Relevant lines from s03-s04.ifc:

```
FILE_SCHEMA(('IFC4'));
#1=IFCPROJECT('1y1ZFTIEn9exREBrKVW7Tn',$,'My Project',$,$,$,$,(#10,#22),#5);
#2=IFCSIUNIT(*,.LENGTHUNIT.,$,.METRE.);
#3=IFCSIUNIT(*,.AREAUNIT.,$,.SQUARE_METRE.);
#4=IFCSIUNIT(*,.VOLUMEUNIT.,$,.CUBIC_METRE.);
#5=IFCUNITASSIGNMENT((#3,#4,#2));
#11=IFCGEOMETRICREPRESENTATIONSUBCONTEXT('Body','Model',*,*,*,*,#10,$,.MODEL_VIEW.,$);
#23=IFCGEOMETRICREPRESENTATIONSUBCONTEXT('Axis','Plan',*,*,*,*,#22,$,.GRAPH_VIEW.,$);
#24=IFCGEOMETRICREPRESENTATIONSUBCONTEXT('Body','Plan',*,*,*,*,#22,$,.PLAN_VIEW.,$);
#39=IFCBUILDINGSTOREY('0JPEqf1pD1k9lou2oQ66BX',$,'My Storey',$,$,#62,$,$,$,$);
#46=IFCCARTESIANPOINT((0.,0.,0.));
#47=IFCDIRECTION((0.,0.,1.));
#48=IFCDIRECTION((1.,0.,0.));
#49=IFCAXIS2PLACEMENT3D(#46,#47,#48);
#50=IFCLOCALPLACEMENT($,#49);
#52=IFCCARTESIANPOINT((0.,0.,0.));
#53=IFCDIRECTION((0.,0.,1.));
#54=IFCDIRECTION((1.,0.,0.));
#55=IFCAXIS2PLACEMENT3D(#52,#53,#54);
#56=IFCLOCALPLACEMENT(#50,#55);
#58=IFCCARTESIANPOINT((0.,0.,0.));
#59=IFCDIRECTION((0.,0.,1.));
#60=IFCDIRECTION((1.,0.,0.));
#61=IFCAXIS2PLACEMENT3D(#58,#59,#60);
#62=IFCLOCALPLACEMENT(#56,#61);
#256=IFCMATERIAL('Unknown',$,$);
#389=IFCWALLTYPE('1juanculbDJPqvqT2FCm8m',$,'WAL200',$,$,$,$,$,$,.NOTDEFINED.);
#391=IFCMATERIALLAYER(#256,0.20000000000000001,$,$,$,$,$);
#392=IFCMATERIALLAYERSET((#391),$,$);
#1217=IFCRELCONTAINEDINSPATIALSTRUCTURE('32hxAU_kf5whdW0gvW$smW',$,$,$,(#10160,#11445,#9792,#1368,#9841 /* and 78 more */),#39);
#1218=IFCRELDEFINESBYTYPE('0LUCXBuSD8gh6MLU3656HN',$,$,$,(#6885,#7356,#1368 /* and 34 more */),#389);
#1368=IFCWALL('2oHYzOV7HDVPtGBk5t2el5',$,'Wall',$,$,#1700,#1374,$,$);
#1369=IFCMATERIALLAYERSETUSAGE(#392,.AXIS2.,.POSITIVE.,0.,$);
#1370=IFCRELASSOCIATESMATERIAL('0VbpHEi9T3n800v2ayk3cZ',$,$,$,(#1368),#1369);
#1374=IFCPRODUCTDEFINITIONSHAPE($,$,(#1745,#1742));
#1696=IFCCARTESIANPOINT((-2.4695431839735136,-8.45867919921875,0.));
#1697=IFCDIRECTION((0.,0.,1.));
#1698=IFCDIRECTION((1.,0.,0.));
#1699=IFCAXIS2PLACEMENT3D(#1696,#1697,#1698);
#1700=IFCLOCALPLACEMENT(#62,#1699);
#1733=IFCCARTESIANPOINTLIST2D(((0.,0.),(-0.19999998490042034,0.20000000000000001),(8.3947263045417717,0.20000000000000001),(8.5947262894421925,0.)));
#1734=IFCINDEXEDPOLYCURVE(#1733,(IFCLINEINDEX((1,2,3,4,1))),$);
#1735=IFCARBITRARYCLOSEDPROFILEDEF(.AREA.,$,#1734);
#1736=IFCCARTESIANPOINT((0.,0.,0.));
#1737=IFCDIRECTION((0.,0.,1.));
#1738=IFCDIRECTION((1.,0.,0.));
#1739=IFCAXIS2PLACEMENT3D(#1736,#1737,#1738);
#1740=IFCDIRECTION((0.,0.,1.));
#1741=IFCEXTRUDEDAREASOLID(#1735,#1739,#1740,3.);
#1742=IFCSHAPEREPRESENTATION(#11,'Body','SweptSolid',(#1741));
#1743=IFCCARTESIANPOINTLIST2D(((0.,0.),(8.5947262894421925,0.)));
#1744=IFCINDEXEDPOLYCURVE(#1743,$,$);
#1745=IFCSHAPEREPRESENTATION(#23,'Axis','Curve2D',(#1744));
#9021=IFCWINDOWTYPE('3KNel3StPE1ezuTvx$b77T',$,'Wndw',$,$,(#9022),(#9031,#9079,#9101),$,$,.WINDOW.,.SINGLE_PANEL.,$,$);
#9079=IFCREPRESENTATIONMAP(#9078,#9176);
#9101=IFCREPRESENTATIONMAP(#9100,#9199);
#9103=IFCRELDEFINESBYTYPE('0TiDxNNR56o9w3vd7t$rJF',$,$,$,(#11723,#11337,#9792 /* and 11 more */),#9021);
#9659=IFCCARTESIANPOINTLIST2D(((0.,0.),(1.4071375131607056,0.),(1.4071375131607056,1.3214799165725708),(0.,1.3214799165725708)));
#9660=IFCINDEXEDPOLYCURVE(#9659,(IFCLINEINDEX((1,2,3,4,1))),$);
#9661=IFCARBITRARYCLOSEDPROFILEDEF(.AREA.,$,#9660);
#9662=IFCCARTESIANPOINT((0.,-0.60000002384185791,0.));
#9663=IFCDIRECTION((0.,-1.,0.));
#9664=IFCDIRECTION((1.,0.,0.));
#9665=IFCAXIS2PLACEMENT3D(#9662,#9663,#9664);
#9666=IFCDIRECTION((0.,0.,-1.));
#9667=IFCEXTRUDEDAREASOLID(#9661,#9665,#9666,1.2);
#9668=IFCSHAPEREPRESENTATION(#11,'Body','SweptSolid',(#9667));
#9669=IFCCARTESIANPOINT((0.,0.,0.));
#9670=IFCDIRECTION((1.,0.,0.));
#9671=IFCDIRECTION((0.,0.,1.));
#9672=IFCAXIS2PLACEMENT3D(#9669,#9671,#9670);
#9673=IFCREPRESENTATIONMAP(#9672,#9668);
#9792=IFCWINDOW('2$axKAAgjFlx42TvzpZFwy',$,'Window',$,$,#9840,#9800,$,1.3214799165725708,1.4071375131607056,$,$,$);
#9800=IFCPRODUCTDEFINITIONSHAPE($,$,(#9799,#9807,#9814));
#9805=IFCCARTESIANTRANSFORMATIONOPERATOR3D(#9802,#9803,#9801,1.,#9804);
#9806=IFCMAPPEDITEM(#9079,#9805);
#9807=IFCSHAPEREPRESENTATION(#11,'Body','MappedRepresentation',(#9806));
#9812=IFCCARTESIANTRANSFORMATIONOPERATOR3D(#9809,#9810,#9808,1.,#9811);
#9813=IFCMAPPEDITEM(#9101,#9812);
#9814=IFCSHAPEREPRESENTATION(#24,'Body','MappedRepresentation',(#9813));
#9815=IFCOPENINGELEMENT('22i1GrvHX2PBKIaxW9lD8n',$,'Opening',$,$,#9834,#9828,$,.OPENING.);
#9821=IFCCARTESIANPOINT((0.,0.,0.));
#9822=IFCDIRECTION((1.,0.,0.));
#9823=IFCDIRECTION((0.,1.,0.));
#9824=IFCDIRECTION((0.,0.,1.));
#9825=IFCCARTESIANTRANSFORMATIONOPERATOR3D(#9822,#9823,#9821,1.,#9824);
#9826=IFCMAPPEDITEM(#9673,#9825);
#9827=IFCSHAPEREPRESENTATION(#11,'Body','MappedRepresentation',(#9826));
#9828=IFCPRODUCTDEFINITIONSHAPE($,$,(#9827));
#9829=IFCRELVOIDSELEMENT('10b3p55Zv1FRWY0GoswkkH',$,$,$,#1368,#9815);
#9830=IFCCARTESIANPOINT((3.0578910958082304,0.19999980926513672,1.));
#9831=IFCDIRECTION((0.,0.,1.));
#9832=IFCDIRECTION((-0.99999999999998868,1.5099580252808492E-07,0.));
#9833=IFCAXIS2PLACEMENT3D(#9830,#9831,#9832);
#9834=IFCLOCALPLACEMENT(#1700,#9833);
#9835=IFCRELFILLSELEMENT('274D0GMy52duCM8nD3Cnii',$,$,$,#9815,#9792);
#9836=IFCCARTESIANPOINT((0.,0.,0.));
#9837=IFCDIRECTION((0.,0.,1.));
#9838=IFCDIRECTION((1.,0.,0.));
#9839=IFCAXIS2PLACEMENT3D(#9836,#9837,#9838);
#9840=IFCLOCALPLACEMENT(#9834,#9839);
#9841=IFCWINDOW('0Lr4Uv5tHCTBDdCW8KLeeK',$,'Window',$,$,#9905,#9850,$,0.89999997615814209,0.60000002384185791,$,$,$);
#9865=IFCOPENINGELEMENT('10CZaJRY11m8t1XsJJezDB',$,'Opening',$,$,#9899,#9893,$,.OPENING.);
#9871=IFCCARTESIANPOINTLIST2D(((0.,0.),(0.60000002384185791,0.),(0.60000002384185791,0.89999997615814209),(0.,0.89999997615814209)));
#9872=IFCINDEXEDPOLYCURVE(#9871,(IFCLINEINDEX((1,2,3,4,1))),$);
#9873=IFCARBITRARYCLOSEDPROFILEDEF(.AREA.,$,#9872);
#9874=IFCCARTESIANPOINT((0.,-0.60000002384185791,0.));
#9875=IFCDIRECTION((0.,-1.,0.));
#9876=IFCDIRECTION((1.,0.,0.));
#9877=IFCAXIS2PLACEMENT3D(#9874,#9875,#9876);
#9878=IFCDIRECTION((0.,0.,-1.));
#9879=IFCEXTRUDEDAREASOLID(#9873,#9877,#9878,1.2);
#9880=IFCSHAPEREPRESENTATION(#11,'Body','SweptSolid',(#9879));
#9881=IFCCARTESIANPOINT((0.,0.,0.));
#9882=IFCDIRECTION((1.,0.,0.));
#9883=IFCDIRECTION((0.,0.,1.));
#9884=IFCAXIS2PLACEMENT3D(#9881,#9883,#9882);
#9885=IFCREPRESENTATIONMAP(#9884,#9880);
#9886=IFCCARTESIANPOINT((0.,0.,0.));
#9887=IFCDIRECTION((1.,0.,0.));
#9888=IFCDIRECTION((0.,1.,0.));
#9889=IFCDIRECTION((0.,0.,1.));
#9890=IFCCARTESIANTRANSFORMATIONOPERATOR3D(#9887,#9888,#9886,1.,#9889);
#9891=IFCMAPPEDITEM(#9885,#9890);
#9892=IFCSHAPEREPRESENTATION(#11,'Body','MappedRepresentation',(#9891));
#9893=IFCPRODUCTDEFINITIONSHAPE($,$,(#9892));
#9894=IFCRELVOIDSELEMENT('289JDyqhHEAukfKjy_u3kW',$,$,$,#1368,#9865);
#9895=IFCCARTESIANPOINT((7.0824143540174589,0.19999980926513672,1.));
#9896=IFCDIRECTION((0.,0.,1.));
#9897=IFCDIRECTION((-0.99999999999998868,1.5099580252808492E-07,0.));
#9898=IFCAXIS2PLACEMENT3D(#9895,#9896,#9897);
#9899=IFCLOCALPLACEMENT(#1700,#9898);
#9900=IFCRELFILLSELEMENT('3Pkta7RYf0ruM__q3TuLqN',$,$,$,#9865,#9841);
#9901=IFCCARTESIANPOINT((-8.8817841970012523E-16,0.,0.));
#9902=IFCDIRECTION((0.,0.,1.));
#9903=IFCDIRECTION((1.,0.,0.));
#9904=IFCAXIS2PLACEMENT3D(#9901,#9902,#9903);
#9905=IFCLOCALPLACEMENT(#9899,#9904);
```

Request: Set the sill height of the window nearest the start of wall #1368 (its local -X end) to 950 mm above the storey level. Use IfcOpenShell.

```python
import numpy as np
import ifcopenshell
import ifcopenshell.api.geometry
import ifcopenshell.geom
import ifcopenshell.util.element
import ifcopenshell.util.placement
import ifcopenshell.util.shape
import ifcopenshell.util.unit

model = ifcopenshell.open("s03-s04.ifc")
unit_scale = ifcopenshell.util.unit.calculate_unit_scale(model)

window = model.by_guid("2$axKAAgjFlx42TvzpZFwy")
opening = window.FillsVoids[0].RelatingOpeningElement
storey = ifcopenshell.util.element.get_container(window, ifc_class="IfcBuildingStorey")
level = ifcopenshell.util.placement.get_local_placement(storey.ObjectPlacement)[2, 3]

# The opening's origin need not be at the sill, so measure its lowest point.
shape = ifcopenshell.geom.create_shape(ifcopenshell.geom.settings(), opening)
bottom = ifcopenshell.util.shape.get_shape_bottom_elevation(shape, shape.geometry) / unit_scale
dz = level + 0.95 - bottom

shift = np.array([0.0, 0.0, dz])
# The window is placed relative to its opening, so it follows when the opening moves.
matrix = ifcopenshell.util.placement.get_local_placement(opening.ObjectPlacement)
matrix[:3, 3] += shift
ifcopenshell.api.geometry.edit_object_placement(
    model, product=opening, matrix=matrix, is_si=False, should_transform_children=True
)

print(f"moved by {dz * unit_scale:+.3f} m")

model.write("s03-s04_updated.ifc")
```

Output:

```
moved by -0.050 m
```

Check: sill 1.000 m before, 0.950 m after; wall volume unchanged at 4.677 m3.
